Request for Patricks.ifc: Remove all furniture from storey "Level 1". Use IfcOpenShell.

First a look at what the model holds.

```python
import ifcopenshell
import ifcopenshell.util.element

model = ifcopenshell.open("Patricks.ifc")
print(model.schema)
storey = next(s for s in model.by_type("IfcBuildingStorey") if s.Name == "Level 1")
furniture = [e for e in ifcopenshell.util.element.get_decomposition(storey) if e.is_a("IfcFurnishingElement")]
seen = {}
for e in furniture:
    element_type = ifcopenshell.util.element.get_type(e)
    name = element_type.Name if element_type not in (None, e) else None
    seen[name] = seen.get(name, 0) + 1
for name, count in sorted(seen.items(), key=str):
    print(count, "x", name)
```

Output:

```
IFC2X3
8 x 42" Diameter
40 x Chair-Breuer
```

```python
import ifcopenshell
import ifcopenshell.api.root
import ifcopenshell.util.element

model = ifcopenshell.open("Patricks.ifc")

storey = next(s for s in model.by_type("IfcBuildingStorey") if s.Name == "Level 1")
furniture = [e for e in ifcopenshell.util.element.get_decomposition(storey) if e.is_a("IfcFurnishingElement")]

for e in furniture:
    ifcopenshell.api.root.remove_product(model, product=e)
print(len(furniture), "removed")

model.write("Patricks_v2.ifc")
```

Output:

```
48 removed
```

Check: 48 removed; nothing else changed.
